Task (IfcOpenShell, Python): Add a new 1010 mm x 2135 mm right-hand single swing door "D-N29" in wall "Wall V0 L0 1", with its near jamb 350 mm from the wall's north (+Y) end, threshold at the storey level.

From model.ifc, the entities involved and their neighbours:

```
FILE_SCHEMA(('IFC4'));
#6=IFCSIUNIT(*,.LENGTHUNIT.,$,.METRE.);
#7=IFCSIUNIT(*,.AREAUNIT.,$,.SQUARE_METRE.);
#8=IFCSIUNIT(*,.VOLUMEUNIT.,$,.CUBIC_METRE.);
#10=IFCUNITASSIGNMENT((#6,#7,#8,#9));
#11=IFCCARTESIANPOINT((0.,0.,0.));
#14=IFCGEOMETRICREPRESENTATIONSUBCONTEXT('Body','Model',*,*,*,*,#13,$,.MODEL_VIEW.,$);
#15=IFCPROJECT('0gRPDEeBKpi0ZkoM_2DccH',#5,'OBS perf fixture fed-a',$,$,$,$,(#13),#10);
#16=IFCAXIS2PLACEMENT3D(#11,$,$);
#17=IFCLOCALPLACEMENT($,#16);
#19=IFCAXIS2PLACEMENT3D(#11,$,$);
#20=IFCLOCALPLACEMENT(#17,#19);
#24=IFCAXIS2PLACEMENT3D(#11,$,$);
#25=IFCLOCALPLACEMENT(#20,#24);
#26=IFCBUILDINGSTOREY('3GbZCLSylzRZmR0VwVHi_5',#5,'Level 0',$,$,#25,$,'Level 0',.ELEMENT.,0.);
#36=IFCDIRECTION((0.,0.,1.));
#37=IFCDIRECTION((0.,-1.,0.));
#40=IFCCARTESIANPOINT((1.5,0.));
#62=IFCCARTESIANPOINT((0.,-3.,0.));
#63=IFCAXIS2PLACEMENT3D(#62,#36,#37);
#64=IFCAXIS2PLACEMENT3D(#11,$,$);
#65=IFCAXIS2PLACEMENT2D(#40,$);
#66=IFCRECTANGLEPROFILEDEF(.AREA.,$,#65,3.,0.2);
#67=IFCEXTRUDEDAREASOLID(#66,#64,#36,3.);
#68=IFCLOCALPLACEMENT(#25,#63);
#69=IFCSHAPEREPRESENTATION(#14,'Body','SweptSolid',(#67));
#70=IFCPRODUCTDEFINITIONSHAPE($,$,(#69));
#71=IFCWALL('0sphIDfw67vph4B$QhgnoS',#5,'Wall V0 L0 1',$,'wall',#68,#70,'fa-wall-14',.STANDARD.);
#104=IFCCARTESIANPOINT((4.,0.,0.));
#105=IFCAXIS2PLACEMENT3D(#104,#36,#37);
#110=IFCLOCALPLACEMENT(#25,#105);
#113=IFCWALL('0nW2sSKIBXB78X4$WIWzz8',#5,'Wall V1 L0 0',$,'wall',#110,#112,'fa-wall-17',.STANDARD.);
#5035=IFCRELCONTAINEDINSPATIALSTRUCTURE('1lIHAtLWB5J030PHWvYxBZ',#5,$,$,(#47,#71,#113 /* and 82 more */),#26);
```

```python
import numpy as np
import ifcopenshell
import ifcopenshell.api.feature
import ifcopenshell.api.geometry
import ifcopenshell.api.root
import ifcopenshell.api.spatial
import ifcopenshell.geom
import ifcopenshell.util.element
import ifcopenshell.util.placement
import ifcopenshell.util.representation
import ifcopenshell.util.shape
import ifcopenshell.util.unit

model = ifcopenshell.open("model.ifc")
unit_scale = ifcopenshell.util.unit.calculate_unit_scale(model)
settings = ifcopenshell.geom.settings()


def volume(element):
    """Net volume in cubic metres, openings subtracted."""
    shape = ifcopenshell.geom.create_shape(settings, element)
    return ifcopenshell.util.shape.get_volume(shape.geometry)


wall = model.by_guid("0sphIDfw67vph4B$QhgnoS")
storey = ifcopenshell.util.element.get_container(wall, ifc_class="IfcBuildingStorey")
context = ifcopenshell.util.representation.get_context(model, "Model", "Body", "MODEL_VIEW")
before = volume(wall)

width, height, from_end, sill = 1.01, 2.135, 0.35, 0.0  # metres

# The wall runs along its own X axis, and the end named is its -X end.
wall_shape = ifcopenshell.geom.create_shape(settings, wall)
x, y, z = ifcopenshell.util.shape.get_vertices(wall_shape.geometry).T
start = x.min() + from_end
face, thickness = float(y.min()), float(y.max() - y.min())
wall_matrix = ifcopenshell.util.placement.get_local_placement(wall.ObjectPlacement)
level = ifcopenshell.util.placement.get_local_placement(storey.ObjectPlacement)[2, 3]


def in_wall(x, y):
    """Placement at x, y metres in the wall's axes, at sill height."""
    matrix = wall_matrix.copy()
    matrix[:, 3] = wall_matrix @ np.array([x / unit_scale, y / unit_scale, 0.0, 1.0])
    matrix[2, 3] = level + sill / unit_scale
    return matrix


# Opening: a box that overshoots both wall faces by 50 mm.
opening = ifcopenshell.api.root.create_entity(model, ifc_class="IfcOpeningElement", predefined_type="OPENING")
box = ifcopenshell.api.geometry.add_wall_representation(
    model, context=context, length=width, height=height, thickness=thickness + 0.1
)
ifcopenshell.api.geometry.assign_representation(model, product=opening, representation=box)
ifcopenshell.api.geometry.edit_object_placement(model, product=opening, matrix=in_wall(start, face - 0.05), is_si=False)
ifcopenshell.api.feature.add_feature(model, feature=opening, element=wall)

door = ifcopenshell.api.root.create_entity(model, ifc_class="IfcDoor", name="D-N29", predefined_type="DOOR")
door.OverallWidth, door.OverallHeight = width / unit_scale, height / unit_scale
door.OperationType = "SINGLE_SWING_RIGHT"
body = ifcopenshell.api.geometry.add_door_representation(
    model,
    context=context,
    overall_width=door.OverallWidth,
    overall_height=door.OverallHeight,
    operation_type="SINGLE_SWING_RIGHT",
    lining_properties={"LiningDepth": thickness / unit_scale, "ThresholdDepth": thickness / unit_scale},
)
ifcopenshell.api.geometry.assign_representation(model, product=door, representation=body)
ifcopenshell.api.spatial.assign_container(model, products=[door], relating_structure=storey)
ifcopenshell.api.feature.add_filling(model, opening=opening, element=door)

# The lining spans the wall, so the door starts at the wall face.
ifcopenshell.api.geometry.edit_object_placement(model, product=door, matrix=in_wall(start, face), is_si=False)

after = volume(wall)

print(f"wall volume {before:.3f} -> {after:.3f} m3")

model.write("model_updated.ifc")
```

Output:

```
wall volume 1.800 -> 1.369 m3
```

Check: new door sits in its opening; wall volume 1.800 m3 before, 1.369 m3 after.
